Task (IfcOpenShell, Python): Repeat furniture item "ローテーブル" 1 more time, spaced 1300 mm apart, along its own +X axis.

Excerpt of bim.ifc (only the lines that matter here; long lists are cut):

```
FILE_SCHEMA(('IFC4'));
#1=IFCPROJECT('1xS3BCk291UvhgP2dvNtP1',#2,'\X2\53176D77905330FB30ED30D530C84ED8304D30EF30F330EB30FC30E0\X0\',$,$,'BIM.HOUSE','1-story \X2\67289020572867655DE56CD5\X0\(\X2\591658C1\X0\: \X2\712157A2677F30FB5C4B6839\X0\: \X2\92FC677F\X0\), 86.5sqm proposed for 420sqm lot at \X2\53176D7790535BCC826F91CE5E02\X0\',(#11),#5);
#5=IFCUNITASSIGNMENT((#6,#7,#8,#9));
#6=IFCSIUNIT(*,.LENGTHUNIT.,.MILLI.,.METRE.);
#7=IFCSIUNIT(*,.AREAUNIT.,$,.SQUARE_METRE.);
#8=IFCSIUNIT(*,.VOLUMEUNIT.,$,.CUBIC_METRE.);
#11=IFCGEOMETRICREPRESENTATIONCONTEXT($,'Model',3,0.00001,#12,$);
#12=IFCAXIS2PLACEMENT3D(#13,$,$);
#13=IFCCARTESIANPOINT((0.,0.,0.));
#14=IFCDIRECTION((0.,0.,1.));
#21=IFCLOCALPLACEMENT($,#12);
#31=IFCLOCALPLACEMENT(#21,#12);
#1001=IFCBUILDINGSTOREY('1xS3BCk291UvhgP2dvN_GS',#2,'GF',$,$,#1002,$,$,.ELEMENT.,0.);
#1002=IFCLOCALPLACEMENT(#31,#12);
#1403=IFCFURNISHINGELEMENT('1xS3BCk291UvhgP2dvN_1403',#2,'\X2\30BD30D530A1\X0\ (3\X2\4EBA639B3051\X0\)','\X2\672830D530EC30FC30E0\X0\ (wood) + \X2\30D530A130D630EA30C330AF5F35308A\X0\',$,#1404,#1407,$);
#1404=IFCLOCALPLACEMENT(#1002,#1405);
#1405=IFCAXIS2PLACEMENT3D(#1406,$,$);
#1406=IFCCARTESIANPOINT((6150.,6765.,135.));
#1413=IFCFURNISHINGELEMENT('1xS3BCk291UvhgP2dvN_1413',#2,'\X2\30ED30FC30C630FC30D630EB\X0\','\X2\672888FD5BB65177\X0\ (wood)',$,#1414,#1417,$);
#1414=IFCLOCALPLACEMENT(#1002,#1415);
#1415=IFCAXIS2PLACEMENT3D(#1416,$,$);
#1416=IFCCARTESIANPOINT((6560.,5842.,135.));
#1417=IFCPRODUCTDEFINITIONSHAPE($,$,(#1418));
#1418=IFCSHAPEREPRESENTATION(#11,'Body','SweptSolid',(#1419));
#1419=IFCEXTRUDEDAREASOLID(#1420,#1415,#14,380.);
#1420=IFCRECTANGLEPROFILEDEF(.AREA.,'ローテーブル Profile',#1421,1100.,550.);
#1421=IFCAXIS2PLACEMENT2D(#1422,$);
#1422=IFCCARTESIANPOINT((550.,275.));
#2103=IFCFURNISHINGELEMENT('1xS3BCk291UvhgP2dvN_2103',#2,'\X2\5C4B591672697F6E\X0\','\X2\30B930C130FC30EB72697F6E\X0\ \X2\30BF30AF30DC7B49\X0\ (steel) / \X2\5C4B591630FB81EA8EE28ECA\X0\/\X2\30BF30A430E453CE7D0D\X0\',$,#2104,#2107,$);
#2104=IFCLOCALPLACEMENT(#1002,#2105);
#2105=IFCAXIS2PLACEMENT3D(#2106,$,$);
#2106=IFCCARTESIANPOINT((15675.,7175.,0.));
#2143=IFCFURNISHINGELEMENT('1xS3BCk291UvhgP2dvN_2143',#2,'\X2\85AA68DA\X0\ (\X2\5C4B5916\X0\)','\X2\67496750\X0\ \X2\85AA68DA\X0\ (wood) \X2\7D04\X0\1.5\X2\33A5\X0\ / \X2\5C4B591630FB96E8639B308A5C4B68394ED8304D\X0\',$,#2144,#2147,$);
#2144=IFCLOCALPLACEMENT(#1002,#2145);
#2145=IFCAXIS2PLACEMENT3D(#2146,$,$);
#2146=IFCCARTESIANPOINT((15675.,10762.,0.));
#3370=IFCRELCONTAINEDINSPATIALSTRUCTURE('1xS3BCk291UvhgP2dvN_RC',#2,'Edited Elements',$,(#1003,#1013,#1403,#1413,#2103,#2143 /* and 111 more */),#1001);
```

```python
import ifcopenshell
import ifcopenshell.api.geometry
import ifcopenshell.api.root
import ifcopenshell.util.element
import ifcopenshell.util.placement

model = ifcopenshell.open("bim.ifc")


def reuse_history(source, copy):
    """copy_class also copies each property set's owner history, people and application; keep the originals."""
    for rel in copy.IsDefinedBy:
        if rel.is_a("IfcRelDefinesByProperties") and (history := rel.RelatingPropertyDefinition.OwnerHistory):
            rel.RelatingPropertyDefinition.OwnerHistory = source.OwnerHistory
            ifcopenshell.util.element.remove_deep2(model, history)


source = model.by_id(1413)
base = ifcopenshell.util.placement.get_local_placement(source.ObjectPlacement)
step = base[:3, 0] * 1300.0

for i in range(1, 2):
    copy = ifcopenshell.api.root.copy_class(model, product=source)
    copy.Representation = ifcopenshell.util.element.copy_deep(
        model, source.Representation, exclude=["IfcGeometricRepresentationContext", "IfcRepresentationMap"]
    )
    reuse_history(source, copy)
    matrix = base.copy()
    matrix[:3, 3] += i * step
    print("added at", matrix[:3, 3].round(3) + 0.0)
    ifcopenshell.api.geometry.edit_object_placement(model, product=copy, matrix=matrix, is_si=False)

model.write("bim_v2.ifc")
```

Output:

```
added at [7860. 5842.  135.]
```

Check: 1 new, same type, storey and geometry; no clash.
